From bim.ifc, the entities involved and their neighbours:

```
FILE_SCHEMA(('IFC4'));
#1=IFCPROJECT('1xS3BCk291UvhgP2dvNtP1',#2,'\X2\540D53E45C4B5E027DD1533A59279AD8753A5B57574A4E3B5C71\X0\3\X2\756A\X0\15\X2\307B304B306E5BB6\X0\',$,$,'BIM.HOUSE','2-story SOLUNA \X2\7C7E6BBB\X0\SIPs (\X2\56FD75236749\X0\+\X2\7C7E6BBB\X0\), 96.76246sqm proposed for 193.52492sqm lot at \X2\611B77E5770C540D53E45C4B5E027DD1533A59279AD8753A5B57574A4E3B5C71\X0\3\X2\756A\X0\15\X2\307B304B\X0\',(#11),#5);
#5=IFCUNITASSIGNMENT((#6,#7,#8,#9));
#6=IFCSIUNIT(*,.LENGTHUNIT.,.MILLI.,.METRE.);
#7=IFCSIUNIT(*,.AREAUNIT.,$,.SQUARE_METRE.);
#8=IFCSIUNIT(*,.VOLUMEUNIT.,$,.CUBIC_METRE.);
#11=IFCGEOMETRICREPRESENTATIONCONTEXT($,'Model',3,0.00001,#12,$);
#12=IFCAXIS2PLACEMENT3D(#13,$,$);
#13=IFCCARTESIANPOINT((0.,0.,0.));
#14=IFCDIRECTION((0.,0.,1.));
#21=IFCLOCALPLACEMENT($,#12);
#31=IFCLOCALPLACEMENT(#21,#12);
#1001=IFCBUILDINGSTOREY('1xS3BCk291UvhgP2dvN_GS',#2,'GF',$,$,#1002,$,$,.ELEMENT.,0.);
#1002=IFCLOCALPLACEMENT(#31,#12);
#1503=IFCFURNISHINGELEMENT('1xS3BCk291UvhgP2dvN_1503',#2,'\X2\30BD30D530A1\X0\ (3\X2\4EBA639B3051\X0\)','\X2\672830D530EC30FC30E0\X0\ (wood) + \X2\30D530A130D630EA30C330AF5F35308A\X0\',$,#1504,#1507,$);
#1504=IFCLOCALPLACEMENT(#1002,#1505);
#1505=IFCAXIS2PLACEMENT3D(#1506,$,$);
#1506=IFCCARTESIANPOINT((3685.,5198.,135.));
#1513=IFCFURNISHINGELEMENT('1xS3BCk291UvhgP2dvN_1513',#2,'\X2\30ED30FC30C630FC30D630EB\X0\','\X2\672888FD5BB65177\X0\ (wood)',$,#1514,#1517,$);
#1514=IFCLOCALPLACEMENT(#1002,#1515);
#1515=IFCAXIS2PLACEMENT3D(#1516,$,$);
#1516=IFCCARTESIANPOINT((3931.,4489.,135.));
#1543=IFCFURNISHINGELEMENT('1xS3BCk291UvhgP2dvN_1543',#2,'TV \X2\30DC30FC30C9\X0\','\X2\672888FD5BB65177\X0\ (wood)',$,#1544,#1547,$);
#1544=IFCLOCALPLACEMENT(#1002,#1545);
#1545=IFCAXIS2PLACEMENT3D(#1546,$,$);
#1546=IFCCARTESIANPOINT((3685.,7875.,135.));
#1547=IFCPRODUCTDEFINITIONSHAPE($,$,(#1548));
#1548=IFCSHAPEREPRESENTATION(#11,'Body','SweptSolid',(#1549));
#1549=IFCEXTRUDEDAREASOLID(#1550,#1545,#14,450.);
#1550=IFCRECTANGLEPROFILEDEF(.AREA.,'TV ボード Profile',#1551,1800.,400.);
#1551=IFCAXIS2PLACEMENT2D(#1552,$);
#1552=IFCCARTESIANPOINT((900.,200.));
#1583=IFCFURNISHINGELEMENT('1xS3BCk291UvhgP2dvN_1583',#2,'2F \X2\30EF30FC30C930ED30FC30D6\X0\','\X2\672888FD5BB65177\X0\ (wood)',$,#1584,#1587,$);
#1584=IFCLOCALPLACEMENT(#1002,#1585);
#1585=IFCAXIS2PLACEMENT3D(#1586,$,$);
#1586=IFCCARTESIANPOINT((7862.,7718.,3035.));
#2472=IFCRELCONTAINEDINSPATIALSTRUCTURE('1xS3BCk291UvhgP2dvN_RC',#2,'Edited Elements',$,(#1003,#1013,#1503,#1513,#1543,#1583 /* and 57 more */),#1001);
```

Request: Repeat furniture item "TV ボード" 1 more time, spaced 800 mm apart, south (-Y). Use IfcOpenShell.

```python
import numpy as np
import ifcopenshell
import ifcopenshell.api.geometry
import ifcopenshell.api.root
import ifcopenshell.util.element
import ifcopenshell.util.placement

model = ifcopenshell.open("bim.ifc")


def reuse_history(source, copy):
    """copy_class also copies each property set's owner history, people and application; keep the originals."""
    for rel in copy.IsDefinedBy:
        if rel.is_a("IfcRelDefinesByProperties") and (history := rel.RelatingPropertyDefinition.OwnerHistory):
            rel.RelatingPropertyDefinition.OwnerHistory = source.OwnerHistory
            ifcopenshell.util.element.remove_deep2(model, history)


source = model.by_id(1543)
base = ifcopenshell.util.placement.get_local_placement(source.ObjectPlacement)
step = np.array([0.0, -1.0, 0.0]) * 800.0

for i in range(1, 2):
    copy = ifcopenshell.api.root.copy_class(model, product=source)
    copy.Representation = ifcopenshell.util.element.copy_deep(
        model, source.Representation, exclude=["IfcGeometricRepresentationContext", "IfcRepresentationMap"]
    )
    reuse_history(source, copy)
    matrix = base.copy()
    matrix[:3, 3] += i * step
    print("added at", matrix[:3, 3].round(3) + 0.0)
    ifcopenshell.api.geometry.edit_object_placement(model, product=copy, matrix=matrix, is_si=False)

model.write("bim_updated.ifc")
```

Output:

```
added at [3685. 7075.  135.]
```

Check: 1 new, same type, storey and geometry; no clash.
